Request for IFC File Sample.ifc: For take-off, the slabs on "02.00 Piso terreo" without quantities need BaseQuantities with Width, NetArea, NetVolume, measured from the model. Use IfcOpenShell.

First a look at what the model holds.

```python
import ifcopenshell
import ifcopenshell.util.element
import ifcopenshell.util.unit

model = ifcopenshell.open("IFC File Sample.ifc")
print(model.schema)
for unit_type in ("LENGTHUNIT", "AREAUNIT", "VOLUMEUNIT"):
    print(unit_type, ifcopenshell.util.unit.calculate_unit_scale(model, unit_type))
storey = next(s for s in model.by_type("IfcBuildingStorey") if s.Name == "02.00 Piso terreo")
slabs = [e for e in ifcopenshell.util.element.get_decomposition(storey) if e.is_a("IfcSlab")]
for e in sorted(slabs, key=lambda e: e.id()):
    print(e.id(), e.is_a(), e.Name, list(ifcopenshell.util.element.get_psets(e, qtos_only=True)), sep=" | ")
```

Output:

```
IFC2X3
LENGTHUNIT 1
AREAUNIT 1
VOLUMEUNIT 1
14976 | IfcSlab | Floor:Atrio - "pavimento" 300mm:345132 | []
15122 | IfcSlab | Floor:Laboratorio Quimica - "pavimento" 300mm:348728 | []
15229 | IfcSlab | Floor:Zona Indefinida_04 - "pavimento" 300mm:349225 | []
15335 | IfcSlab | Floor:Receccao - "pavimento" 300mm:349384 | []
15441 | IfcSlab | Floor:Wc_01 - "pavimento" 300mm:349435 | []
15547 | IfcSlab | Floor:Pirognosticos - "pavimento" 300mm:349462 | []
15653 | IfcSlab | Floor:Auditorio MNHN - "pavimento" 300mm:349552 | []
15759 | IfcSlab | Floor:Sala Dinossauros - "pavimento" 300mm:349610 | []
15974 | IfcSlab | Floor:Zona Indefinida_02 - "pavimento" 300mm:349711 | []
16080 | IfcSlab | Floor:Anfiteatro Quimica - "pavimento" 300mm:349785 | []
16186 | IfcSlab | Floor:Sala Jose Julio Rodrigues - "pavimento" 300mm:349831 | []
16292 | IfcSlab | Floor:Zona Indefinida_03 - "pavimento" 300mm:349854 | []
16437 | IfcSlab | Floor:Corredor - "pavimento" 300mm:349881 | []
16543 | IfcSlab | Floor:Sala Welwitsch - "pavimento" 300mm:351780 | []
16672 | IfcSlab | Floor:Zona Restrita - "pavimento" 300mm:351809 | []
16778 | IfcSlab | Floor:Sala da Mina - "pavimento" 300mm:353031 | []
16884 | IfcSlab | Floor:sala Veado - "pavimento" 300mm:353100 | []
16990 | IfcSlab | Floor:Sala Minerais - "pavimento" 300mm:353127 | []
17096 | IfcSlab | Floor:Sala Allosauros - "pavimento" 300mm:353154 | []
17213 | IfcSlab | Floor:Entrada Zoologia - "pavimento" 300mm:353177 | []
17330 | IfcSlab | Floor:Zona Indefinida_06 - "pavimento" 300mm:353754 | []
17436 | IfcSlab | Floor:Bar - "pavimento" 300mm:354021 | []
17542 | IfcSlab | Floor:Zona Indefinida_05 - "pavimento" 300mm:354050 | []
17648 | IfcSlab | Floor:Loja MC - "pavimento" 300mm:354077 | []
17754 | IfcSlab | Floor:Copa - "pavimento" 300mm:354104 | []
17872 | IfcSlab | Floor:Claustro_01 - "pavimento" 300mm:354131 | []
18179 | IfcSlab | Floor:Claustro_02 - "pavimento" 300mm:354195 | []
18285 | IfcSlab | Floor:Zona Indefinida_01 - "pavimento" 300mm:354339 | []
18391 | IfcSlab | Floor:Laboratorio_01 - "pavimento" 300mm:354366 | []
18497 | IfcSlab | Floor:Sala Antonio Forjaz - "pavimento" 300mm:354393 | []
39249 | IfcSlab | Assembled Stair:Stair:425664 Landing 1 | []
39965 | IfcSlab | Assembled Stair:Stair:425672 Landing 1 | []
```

```python
import ifcopenshell
import ifcopenshell.api.pset
import ifcopenshell.geom
import ifcopenshell.util.element
import ifcopenshell.util.shape
import ifcopenshell.util.unit

model = ifcopenshell.open("IFC File Sample.ifc")
unit_scale = ifcopenshell.util.unit.calculate_unit_scale(model)
area_scale = ifcopenshell.util.unit.calculate_unit_scale(model, "AREAUNIT")
volume_scale = ifcopenshell.util.unit.calculate_unit_scale(model, "VOLUMEUNIT")
settings = ifcopenshell.geom.settings()

storey = next(s for s in model.by_type("IfcBuildingStorey") if s.Name == "02.00 Piso terreo")
slabs = [e for e in ifcopenshell.util.element.get_decomposition(storey) if e.is_a("IfcSlab")]

for e in sorted(slabs, key=lambda e: e.id()):
    if ifcopenshell.util.element.get_psets(e, qtos_only=True, should_inherit=False):
        continue
    # Geometry comes back in metres, in the element's own axes.
    shape = ifcopenshell.geom.create_shape(settings, e)
    values = {
        "Width": ifcopenshell.util.shape.get_z(shape.geometry) / unit_scale,
        "NetArea": ifcopenshell.util.shape.get_footprint_area(shape.geometry) / area_scale,
        "NetVolume": ifcopenshell.util.shape.get_volume(shape.geometry) / volume_scale,
    }
    qto = ifcopenshell.api.pset.add_qto(model, product=e, name="BaseQuantities")
    ifcopenshell.api.pset.edit_qto(model, qto=qto, properties=values)
    print(e.id(), {k: round(v, 3) for k, v in values.items()})

model.write("IFC File Sample_v2.ifc")
```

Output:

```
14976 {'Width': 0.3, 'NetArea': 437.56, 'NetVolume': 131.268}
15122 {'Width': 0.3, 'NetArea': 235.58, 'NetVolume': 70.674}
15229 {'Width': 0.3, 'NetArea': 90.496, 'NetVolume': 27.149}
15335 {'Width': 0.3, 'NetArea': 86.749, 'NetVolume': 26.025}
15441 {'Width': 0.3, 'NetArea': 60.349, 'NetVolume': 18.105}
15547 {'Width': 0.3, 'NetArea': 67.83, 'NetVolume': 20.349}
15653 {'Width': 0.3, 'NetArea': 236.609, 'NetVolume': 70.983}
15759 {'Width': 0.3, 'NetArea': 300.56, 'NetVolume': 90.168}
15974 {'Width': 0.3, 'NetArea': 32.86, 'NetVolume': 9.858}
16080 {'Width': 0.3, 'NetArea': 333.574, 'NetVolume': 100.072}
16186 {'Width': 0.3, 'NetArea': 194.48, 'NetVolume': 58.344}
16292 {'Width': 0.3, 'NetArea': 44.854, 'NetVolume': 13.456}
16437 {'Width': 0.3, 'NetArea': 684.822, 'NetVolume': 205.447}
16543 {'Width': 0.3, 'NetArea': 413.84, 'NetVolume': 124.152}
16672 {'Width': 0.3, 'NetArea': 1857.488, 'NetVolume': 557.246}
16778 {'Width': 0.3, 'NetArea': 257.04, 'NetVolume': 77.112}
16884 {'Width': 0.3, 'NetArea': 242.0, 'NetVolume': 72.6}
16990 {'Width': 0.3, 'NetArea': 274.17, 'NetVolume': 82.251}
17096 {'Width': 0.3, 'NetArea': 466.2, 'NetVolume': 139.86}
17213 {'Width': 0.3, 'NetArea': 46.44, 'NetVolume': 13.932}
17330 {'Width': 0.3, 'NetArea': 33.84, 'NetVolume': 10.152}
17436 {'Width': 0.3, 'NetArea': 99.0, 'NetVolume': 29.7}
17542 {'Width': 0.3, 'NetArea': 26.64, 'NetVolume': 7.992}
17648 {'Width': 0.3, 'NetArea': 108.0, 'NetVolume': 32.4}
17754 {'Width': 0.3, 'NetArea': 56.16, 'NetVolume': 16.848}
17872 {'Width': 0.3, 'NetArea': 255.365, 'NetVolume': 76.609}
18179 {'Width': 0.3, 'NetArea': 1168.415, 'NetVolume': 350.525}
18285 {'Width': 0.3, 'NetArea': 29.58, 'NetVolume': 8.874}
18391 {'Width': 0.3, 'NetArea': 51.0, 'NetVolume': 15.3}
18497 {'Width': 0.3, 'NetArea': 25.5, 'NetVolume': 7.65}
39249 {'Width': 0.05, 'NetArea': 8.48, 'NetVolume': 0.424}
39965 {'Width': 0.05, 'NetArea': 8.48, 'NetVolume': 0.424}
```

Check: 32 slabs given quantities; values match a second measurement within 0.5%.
